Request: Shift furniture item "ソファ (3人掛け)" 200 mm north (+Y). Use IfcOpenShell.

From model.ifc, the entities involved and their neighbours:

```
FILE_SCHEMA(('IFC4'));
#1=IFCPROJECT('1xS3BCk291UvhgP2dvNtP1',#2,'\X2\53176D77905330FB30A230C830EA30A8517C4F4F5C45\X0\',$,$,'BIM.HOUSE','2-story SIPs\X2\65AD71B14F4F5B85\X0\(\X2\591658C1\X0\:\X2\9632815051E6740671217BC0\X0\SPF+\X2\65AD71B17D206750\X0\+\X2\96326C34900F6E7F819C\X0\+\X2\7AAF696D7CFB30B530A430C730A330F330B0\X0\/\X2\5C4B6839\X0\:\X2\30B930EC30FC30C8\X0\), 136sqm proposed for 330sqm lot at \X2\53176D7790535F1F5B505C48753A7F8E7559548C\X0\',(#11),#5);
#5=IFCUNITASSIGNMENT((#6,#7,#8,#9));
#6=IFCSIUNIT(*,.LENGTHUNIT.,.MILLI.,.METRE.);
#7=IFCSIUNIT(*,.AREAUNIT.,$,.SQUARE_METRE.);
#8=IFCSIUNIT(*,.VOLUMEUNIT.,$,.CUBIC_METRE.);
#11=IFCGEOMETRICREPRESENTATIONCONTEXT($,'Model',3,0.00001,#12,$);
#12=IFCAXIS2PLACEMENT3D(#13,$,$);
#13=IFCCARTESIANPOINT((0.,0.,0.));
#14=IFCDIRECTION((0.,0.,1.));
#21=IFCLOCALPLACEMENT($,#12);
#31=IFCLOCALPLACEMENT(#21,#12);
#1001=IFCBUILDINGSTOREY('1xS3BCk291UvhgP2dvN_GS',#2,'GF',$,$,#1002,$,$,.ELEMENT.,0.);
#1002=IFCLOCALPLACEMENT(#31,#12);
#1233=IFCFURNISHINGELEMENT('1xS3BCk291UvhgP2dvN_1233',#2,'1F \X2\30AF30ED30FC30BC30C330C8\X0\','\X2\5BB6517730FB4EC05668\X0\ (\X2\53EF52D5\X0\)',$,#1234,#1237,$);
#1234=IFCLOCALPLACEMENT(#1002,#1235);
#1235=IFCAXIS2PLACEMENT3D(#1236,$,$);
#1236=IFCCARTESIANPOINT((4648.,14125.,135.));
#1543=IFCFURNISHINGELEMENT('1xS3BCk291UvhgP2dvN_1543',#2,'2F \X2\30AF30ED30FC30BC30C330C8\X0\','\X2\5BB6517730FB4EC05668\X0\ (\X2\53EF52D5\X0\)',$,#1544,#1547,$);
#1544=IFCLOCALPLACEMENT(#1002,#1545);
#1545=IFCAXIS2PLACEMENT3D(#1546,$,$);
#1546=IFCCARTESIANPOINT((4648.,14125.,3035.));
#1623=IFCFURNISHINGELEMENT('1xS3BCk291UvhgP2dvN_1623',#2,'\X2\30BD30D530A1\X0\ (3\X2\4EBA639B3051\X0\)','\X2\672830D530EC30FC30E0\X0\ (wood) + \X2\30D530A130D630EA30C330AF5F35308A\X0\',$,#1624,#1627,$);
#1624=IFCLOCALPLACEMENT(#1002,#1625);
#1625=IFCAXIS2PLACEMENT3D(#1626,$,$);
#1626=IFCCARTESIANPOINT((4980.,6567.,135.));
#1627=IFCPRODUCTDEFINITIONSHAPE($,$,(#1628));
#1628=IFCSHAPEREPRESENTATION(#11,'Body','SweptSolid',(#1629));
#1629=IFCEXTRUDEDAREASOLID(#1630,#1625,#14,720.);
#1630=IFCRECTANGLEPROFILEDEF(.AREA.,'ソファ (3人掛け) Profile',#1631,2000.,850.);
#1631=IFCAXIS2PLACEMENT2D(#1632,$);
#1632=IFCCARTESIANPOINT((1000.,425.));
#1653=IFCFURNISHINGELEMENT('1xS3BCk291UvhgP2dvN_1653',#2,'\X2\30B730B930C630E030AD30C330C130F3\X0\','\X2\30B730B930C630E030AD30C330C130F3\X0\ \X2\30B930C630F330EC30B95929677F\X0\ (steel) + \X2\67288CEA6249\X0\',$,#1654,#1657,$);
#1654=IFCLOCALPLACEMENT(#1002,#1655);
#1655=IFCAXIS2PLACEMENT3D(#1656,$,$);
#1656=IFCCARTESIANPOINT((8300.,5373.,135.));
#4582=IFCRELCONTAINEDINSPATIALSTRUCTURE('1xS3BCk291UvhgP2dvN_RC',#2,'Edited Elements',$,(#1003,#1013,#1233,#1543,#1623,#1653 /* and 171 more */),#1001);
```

```python
import ifcopenshell
import ifcopenshell.api.geometry
import ifcopenshell.util.placement

model = ifcopenshell.open("model.ifc")

item = model.by_id(1623)
matrix = ifcopenshell.util.placement.get_local_placement(item.ObjectPlacement)
matrix[1, 3] += 200.0
ifcopenshell.api.geometry.edit_object_placement(model, product=item, matrix=matrix, is_si=False)

print(ifcopenshell.util.placement.get_local_placement(item.ObjectPlacement).round(3) + 0.0)

model.write("model-out.ifc")
```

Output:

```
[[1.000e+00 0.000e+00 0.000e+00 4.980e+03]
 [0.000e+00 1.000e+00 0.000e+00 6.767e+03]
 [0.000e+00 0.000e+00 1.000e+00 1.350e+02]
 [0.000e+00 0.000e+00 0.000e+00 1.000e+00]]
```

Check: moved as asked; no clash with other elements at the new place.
